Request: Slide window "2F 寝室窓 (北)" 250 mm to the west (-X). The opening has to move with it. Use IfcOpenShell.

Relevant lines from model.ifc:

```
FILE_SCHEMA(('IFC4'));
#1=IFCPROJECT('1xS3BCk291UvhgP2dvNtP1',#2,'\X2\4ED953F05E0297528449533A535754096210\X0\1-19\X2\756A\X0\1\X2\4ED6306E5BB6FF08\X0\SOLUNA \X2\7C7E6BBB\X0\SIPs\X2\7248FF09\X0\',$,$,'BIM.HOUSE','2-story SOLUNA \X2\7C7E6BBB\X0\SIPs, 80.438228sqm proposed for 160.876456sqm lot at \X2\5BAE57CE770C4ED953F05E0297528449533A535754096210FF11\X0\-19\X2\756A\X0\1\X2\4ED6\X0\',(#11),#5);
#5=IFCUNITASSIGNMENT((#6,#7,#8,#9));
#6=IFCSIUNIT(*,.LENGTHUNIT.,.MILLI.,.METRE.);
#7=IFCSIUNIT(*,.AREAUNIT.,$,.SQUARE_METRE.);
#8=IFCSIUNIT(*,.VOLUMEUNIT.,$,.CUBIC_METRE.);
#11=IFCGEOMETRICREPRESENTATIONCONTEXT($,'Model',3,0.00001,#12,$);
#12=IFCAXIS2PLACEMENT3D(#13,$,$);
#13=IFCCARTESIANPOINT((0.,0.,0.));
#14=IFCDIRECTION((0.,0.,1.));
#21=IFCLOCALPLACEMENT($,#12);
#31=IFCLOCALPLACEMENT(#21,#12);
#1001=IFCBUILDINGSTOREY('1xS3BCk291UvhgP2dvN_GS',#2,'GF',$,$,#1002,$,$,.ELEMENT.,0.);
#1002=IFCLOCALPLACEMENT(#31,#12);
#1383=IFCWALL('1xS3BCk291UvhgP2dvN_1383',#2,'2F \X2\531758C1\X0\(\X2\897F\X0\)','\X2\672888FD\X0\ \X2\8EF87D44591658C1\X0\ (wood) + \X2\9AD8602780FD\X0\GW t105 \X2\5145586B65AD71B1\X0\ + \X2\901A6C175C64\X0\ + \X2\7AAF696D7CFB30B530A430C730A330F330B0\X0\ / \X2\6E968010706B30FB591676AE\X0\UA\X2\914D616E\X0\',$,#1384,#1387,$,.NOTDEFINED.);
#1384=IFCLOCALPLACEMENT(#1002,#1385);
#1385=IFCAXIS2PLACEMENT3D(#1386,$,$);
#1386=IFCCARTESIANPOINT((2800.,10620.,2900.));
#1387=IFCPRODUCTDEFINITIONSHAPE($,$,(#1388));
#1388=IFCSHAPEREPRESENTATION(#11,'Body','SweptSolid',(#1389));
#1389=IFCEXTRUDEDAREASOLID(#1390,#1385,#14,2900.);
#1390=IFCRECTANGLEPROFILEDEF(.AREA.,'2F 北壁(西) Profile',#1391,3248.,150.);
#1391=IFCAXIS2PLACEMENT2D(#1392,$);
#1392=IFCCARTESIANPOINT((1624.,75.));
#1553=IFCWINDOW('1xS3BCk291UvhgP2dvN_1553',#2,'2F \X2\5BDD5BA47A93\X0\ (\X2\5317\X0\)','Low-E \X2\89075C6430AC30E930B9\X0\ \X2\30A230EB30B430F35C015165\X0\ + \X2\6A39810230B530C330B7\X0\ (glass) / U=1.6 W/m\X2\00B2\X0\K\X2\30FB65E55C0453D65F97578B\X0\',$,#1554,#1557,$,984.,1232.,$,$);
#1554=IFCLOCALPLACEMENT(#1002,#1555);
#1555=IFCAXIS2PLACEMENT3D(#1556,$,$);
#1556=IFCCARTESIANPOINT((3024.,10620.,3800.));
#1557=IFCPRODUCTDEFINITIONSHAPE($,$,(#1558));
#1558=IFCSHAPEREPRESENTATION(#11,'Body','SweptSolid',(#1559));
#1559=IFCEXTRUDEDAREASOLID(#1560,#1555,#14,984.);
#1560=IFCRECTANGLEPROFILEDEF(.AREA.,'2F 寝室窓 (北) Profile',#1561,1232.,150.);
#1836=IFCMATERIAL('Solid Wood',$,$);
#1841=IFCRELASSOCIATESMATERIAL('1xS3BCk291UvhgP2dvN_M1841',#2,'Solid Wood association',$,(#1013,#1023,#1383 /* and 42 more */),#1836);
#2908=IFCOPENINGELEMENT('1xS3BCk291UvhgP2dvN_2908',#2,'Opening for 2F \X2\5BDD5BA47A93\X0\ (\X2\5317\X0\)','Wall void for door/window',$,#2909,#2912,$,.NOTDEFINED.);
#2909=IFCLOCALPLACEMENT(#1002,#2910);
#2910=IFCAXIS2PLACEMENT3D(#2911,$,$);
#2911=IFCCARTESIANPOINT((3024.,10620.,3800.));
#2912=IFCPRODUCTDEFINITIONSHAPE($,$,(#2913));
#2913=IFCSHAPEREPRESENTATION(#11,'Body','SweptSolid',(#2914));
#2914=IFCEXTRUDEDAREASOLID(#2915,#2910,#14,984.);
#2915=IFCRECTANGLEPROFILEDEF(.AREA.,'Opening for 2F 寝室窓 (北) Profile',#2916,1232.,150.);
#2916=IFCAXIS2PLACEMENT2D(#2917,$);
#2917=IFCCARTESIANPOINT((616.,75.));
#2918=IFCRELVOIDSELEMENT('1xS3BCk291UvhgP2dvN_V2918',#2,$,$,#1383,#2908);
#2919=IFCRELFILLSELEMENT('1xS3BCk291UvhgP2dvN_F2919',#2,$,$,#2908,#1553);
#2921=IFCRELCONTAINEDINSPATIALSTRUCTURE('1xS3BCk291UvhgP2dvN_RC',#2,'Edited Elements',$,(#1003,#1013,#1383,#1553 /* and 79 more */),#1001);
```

```python
import ifcopenshell
import ifcopenshell.api.geometry
import ifcopenshell.util.placement

model = ifcopenshell.open("model.ifc")

window = model.by_id(1553)
opening = window.FillsVoids[0].RelatingOpeningElement
wall = opening.VoidsElements[0].RelatingBuildingElement

wall_matrix = ifcopenshell.util.placement.get_local_placement(wall.ObjectPlacement)
shift = wall_matrix[:3, 0] * -250.0
before = ifcopenshell.util.placement.get_local_placement(window.ObjectPlacement)[:3, 3].copy()

# The window is not placed relative to its opening, so move both.
for product in (opening, window):
    matrix = ifcopenshell.util.placement.get_local_placement(product.ObjectPlacement)
    matrix[:3, 3] += shift
    ifcopenshell.api.geometry.edit_object_placement(model, product=product, matrix=matrix, is_si=False)

after = ifcopenshell.util.placement.get_local_placement(window.ObjectPlacement)[:3, 3]
print("window moved by", (after - before).round(3) + 0.0)

model.write("model_updated.ifc")
```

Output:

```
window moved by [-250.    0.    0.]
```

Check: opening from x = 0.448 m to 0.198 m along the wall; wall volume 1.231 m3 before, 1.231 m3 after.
